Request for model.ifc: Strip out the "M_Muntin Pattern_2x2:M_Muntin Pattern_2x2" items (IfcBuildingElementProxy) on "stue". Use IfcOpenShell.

First a look at what the model holds.

```python
import ifcopenshell
import ifcopenshell.util.element

model = ifcopenshell.open("model.ifc")
print(model.schema)
storey = next(s for s in model.by_type("IfcBuildingStorey") if s.Name == "stue")
proxies = [e for e in ifcopenshell.util.element.get_decomposition(storey) if e.is_a("IfcBuildingElementProxy")]
seen = {}
for e in proxies:
    element_type = ifcopenshell.util.element.get_type(e)
    name = element_type.Name if element_type not in (None, e) else None
    seen[name] = seen.get(name, 0) + 1
for name, count in sorted(seen.items(), key=str):
    print(count, "x", name)
```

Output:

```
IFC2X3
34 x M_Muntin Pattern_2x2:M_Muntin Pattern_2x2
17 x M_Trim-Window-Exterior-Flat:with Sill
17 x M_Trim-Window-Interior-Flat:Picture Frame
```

```python
import ifcopenshell
import ifcopenshell.api.root
import ifcopenshell.util.element

model = ifcopenshell.open("model.ifc")

storey = next(s for s in model.by_type("IfcBuildingStorey") if s.Name == "stue")
proxies = [e for e in ifcopenshell.util.element.get_decomposition(storey) if e.is_a("IfcBuildingElementProxy")]
targets = [e for e in proxies if (t := ifcopenshell.util.element.get_type(e)) not in (None, e) and t.Name == "M_Muntin Pattern_2x2:M_Muntin Pattern_2x2"]

for e in targets:
    ifcopenshell.api.root.remove_product(model, product=e)
print(len(targets), "removed")

model.write("model_rev.ifc")
```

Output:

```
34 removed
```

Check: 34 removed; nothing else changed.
